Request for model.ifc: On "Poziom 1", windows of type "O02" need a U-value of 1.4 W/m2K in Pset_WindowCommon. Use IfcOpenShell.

First a look at what the model holds.

```python
import ifcopenshell
import ifcopenshell.util.element

model = ifcopenshell.open("model.ifc")
print(model.schema)
storey = next(s for s in model.by_type("IfcBuildingStorey") if s.Name == "Poziom 1")
windows = [e for e in ifcopenshell.util.element.get_decomposition(storey) if e.is_a("IfcWindow")]
seen = {}
for e in windows:
    element_type = ifcopenshell.util.element.get_type(e)
    key = (element_type.Name if element_type != e and element_type else None, ifcopenshell.util.element.get_pset(e, "Pset_WindowCommon", "ThermalTransmittance"))
    seen[key] = seen.get(key, 0) + 1
for (name, value), count in sorted(seen.items(), key=str):
    print(count, "x", name, "|", value)
```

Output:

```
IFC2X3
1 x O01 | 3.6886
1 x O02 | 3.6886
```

```python
import ifcopenshell
import ifcopenshell.api.pset
import ifcopenshell.util.element

model = ifcopenshell.open("model.ifc")

storey = next(s for s in model.by_type("IfcBuildingStorey") if s.Name == "Poziom 1")
windows = [e for e in ifcopenshell.util.element.get_decomposition(storey) if e.is_a("IfcWindow")]

count = 0
for e in windows:
    element_type = ifcopenshell.util.element.get_type(e)
    if element_type in (None, e) or element_type.Name != "O02":
        continue
    # add_pset returns the element's existing set when there is one.
    pset = ifcopenshell.api.pset.add_pset(model, product=e, name="Pset_WindowCommon")
    ifcopenshell.api.pset.edit_pset(model, pset=pset, properties={"ThermalTransmittance": 1.4})
    count += 1

print(count, "windows updated")

model.write("model_updated.ifc")
```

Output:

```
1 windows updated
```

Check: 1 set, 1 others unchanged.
